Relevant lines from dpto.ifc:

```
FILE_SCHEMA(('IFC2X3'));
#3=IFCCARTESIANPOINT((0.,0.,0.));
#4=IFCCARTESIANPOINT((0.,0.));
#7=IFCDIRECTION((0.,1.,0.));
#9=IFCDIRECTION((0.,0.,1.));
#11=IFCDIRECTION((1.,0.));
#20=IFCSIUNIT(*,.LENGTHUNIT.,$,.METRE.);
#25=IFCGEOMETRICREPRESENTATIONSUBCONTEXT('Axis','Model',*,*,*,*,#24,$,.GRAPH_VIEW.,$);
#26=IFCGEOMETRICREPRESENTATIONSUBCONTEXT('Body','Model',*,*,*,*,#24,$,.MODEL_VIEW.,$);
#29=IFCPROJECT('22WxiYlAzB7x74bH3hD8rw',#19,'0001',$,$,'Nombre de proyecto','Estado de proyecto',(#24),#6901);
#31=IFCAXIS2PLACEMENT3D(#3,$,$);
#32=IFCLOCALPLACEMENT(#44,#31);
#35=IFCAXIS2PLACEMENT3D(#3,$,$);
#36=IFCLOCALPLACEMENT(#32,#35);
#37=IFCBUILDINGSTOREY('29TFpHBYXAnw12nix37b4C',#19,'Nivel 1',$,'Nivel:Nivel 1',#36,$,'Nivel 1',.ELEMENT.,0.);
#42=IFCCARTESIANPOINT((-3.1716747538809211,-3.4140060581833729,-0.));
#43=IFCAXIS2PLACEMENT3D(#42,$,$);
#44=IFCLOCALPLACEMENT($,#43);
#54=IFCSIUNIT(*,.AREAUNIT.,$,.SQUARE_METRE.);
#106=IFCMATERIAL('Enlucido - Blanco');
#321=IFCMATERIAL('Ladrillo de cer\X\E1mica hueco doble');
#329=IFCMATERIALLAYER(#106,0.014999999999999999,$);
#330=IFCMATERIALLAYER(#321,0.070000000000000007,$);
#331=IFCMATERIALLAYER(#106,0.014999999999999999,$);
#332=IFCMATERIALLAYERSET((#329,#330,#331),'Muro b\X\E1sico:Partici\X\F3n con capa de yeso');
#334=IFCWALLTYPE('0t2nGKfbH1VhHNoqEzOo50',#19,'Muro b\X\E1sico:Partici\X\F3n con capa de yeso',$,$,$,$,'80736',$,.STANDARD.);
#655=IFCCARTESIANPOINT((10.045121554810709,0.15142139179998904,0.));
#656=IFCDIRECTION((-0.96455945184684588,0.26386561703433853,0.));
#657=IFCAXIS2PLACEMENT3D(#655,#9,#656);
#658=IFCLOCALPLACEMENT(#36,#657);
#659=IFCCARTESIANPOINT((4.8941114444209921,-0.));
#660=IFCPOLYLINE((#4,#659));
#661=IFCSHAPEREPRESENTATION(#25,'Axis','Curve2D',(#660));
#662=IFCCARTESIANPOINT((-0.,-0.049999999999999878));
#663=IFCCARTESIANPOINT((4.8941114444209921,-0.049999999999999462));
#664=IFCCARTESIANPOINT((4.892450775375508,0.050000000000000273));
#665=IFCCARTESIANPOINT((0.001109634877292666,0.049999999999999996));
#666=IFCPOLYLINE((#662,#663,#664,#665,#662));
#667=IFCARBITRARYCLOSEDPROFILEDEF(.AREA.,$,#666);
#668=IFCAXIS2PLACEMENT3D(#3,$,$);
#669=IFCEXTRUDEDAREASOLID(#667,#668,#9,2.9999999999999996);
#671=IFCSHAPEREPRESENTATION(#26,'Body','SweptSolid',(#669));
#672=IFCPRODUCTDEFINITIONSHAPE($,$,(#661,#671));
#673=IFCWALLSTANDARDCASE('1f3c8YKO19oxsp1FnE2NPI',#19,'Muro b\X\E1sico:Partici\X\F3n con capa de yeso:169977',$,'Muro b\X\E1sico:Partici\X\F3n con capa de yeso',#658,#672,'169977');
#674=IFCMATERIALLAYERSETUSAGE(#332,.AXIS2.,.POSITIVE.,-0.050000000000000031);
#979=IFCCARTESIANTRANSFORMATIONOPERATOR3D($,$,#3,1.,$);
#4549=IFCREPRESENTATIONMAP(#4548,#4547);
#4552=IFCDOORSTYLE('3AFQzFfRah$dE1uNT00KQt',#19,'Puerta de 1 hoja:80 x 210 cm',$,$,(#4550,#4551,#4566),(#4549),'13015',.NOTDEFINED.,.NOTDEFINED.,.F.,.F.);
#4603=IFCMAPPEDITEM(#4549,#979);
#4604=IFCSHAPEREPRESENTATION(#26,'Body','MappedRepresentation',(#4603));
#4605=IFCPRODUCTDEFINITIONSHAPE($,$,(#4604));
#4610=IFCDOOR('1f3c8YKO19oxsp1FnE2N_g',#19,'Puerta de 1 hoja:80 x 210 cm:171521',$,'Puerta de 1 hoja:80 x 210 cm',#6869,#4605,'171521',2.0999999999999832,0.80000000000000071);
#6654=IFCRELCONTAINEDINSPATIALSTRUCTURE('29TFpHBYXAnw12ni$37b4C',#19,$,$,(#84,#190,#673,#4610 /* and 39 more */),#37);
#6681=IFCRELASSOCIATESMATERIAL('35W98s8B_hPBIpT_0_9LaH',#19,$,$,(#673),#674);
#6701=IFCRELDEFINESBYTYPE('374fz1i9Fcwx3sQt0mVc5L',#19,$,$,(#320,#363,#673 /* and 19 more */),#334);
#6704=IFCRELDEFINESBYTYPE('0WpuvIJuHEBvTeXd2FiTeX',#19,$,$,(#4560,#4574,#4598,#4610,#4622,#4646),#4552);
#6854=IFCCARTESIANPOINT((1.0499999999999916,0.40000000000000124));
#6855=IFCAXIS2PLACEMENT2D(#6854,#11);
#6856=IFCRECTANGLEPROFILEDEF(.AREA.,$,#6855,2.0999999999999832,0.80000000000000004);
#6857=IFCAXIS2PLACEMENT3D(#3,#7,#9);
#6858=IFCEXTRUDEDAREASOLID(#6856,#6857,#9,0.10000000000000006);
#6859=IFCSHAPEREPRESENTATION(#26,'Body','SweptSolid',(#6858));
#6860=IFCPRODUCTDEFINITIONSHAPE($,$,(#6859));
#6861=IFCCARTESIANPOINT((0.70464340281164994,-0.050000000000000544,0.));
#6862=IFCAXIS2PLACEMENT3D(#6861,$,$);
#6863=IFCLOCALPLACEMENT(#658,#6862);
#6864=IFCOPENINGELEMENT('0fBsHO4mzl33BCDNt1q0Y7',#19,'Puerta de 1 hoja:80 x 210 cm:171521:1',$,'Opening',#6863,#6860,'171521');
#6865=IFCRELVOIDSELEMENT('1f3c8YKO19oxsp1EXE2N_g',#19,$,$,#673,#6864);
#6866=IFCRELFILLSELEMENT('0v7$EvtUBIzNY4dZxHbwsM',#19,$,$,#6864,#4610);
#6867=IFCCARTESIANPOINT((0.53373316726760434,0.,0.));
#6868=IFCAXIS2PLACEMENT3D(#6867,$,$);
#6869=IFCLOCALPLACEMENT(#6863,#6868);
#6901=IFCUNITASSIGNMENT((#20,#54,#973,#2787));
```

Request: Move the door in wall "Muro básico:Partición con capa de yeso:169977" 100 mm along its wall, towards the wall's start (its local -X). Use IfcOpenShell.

```python
import ifcopenshell
import ifcopenshell.api.geometry
import ifcopenshell.util.placement
import ifcopenshell.util.unit

model = ifcopenshell.open("dpto.ifc")
unit_scale = ifcopenshell.util.unit.calculate_unit_scale(model)

door = model.by_guid("1f3c8YKO19oxsp1FnE2N_g")
opening = door.FillsVoids[0].RelatingOpeningElement
wall = opening.VoidsElements[0].RelatingBuildingElement

wall_matrix = ifcopenshell.util.placement.get_local_placement(wall.ObjectPlacement)
shift = wall_matrix[:3, 0] * -0.1 / unit_scale
before = ifcopenshell.util.placement.get_local_placement(door.ObjectPlacement)[:3, 3].copy()

# The door is placed relative to its opening, so it follows when the opening moves.
matrix = ifcopenshell.util.placement.get_local_placement(opening.ObjectPlacement)
matrix[:3, 3] += shift
ifcopenshell.api.geometry.edit_object_placement(
    model, product=opening, matrix=matrix, is_si=False, should_transform_children=True
)

after = ifcopenshell.util.placement.get_local_placement(door.ObjectPlacement)[:3, 3]
print("door moved by", (after - before).round(3) + 0.0)

model.write("dpto-out.ifc")
```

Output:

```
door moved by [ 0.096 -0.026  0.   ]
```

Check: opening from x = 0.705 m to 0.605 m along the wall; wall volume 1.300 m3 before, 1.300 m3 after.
